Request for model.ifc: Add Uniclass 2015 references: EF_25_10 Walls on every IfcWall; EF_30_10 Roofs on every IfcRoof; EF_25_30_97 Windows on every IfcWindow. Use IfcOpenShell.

First a look at what the model holds.

```python
import ifcopenshell

model = ifcopenshell.open("model.ifc")
print(model.schema)
print("classifications:", [c.Name for c in model.by_type("IfcClassification")])
for ifc_class in ("IfcDoor", "IfcRoof", "IfcStair", "IfcWall", "IfcWindow"):
    print(ifc_class, len(model.by_type(ifc_class)))
```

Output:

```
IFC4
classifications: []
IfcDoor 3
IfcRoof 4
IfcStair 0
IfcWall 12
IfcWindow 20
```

```python
import ifcopenshell
import ifcopenshell.api.classification

model = ifcopenshell.open("model.ifc")

system = ifcopenshell.api.classification.add_classification(model, classification="Uniclass 2015")

codes = {
    "IfcWall": ("EF_25_10", "Walls"),
    "IfcRoof": ("EF_30_10", "Roofs"),
    "IfcWindow": ("EF_25_30_97", "Windows"),
}
for ifc_class, (code, name) in codes.items():
    products = model.by_type(ifc_class)
    ifcopenshell.api.classification.add_reference(
        model, products=products, classification=system, identification=code, name=name
    )
    print(code, len(products))

model.write("model_edited.ifc")
```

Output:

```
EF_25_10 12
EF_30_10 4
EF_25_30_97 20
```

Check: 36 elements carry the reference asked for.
